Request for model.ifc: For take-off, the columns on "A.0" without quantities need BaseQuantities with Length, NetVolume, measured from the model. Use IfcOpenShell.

First a look at what the model holds.

```python
import ifcopenshell
import ifcopenshell.util.element
import ifcopenshell.util.unit

model = ifcopenshell.open("model.ifc")
print(model.schema)
for unit_type in ("LENGTHUNIT", "AREAUNIT", "VOLUMEUNIT"):
    print(unit_type, ifcopenshell.util.unit.calculate_unit_scale(model, unit_type))
storey = next(s for s in model.by_type("IfcBuildingStorey") if s.Name == "A.0")
columns = [e for e in ifcopenshell.util.element.get_decomposition(storey) if e.is_a("IfcColumn")]
for e in sorted(columns, key=lambda e: e.id()):
    print(e.id(), e.is_a(), e.Name, list(ifcopenshell.util.element.get_psets(e, qtos_only=True)), sep=" | ")
```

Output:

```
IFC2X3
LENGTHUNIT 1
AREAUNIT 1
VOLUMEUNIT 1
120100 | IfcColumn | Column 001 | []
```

```python
import ifcopenshell
import ifcopenshell.api.pset
import ifcopenshell.geom
import ifcopenshell.util.element
import ifcopenshell.util.shape
import ifcopenshell.util.unit

model = ifcopenshell.open("model.ifc")
unit_scale = ifcopenshell.util.unit.calculate_unit_scale(model)
volume_scale = ifcopenshell.util.unit.calculate_unit_scale(model, "VOLUMEUNIT")
settings = ifcopenshell.geom.settings()

storey = next(s for s in model.by_type("IfcBuildingStorey") if s.Name == "A.0")
columns = [e for e in ifcopenshell.util.element.get_decomposition(storey) if e.is_a("IfcColumn")]

for e in sorted(columns, key=lambda e: e.id()):
    if ifcopenshell.util.element.get_psets(e, qtos_only=True, should_inherit=False):
        continue
    # Geometry comes back in metres, in the element's own axes.
    shape = ifcopenshell.geom.create_shape(settings, e)
    values = {
        "Length": ifcopenshell.util.shape.get_z(shape.geometry) / unit_scale,
        "NetVolume": ifcopenshell.util.shape.get_volume(shape.geometry) / volume_scale,
    }
    qto = ifcopenshell.api.pset.add_qto(model, product=e, name="BaseQuantities")
    ifcopenshell.api.pset.edit_qto(model, qto=qto, properties=values)
    print(e.id(), {k: round(v, 3) for k, v in values.items()})

model.write("model-out.ifc")
```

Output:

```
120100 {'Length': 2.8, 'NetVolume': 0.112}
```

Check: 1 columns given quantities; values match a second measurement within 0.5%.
